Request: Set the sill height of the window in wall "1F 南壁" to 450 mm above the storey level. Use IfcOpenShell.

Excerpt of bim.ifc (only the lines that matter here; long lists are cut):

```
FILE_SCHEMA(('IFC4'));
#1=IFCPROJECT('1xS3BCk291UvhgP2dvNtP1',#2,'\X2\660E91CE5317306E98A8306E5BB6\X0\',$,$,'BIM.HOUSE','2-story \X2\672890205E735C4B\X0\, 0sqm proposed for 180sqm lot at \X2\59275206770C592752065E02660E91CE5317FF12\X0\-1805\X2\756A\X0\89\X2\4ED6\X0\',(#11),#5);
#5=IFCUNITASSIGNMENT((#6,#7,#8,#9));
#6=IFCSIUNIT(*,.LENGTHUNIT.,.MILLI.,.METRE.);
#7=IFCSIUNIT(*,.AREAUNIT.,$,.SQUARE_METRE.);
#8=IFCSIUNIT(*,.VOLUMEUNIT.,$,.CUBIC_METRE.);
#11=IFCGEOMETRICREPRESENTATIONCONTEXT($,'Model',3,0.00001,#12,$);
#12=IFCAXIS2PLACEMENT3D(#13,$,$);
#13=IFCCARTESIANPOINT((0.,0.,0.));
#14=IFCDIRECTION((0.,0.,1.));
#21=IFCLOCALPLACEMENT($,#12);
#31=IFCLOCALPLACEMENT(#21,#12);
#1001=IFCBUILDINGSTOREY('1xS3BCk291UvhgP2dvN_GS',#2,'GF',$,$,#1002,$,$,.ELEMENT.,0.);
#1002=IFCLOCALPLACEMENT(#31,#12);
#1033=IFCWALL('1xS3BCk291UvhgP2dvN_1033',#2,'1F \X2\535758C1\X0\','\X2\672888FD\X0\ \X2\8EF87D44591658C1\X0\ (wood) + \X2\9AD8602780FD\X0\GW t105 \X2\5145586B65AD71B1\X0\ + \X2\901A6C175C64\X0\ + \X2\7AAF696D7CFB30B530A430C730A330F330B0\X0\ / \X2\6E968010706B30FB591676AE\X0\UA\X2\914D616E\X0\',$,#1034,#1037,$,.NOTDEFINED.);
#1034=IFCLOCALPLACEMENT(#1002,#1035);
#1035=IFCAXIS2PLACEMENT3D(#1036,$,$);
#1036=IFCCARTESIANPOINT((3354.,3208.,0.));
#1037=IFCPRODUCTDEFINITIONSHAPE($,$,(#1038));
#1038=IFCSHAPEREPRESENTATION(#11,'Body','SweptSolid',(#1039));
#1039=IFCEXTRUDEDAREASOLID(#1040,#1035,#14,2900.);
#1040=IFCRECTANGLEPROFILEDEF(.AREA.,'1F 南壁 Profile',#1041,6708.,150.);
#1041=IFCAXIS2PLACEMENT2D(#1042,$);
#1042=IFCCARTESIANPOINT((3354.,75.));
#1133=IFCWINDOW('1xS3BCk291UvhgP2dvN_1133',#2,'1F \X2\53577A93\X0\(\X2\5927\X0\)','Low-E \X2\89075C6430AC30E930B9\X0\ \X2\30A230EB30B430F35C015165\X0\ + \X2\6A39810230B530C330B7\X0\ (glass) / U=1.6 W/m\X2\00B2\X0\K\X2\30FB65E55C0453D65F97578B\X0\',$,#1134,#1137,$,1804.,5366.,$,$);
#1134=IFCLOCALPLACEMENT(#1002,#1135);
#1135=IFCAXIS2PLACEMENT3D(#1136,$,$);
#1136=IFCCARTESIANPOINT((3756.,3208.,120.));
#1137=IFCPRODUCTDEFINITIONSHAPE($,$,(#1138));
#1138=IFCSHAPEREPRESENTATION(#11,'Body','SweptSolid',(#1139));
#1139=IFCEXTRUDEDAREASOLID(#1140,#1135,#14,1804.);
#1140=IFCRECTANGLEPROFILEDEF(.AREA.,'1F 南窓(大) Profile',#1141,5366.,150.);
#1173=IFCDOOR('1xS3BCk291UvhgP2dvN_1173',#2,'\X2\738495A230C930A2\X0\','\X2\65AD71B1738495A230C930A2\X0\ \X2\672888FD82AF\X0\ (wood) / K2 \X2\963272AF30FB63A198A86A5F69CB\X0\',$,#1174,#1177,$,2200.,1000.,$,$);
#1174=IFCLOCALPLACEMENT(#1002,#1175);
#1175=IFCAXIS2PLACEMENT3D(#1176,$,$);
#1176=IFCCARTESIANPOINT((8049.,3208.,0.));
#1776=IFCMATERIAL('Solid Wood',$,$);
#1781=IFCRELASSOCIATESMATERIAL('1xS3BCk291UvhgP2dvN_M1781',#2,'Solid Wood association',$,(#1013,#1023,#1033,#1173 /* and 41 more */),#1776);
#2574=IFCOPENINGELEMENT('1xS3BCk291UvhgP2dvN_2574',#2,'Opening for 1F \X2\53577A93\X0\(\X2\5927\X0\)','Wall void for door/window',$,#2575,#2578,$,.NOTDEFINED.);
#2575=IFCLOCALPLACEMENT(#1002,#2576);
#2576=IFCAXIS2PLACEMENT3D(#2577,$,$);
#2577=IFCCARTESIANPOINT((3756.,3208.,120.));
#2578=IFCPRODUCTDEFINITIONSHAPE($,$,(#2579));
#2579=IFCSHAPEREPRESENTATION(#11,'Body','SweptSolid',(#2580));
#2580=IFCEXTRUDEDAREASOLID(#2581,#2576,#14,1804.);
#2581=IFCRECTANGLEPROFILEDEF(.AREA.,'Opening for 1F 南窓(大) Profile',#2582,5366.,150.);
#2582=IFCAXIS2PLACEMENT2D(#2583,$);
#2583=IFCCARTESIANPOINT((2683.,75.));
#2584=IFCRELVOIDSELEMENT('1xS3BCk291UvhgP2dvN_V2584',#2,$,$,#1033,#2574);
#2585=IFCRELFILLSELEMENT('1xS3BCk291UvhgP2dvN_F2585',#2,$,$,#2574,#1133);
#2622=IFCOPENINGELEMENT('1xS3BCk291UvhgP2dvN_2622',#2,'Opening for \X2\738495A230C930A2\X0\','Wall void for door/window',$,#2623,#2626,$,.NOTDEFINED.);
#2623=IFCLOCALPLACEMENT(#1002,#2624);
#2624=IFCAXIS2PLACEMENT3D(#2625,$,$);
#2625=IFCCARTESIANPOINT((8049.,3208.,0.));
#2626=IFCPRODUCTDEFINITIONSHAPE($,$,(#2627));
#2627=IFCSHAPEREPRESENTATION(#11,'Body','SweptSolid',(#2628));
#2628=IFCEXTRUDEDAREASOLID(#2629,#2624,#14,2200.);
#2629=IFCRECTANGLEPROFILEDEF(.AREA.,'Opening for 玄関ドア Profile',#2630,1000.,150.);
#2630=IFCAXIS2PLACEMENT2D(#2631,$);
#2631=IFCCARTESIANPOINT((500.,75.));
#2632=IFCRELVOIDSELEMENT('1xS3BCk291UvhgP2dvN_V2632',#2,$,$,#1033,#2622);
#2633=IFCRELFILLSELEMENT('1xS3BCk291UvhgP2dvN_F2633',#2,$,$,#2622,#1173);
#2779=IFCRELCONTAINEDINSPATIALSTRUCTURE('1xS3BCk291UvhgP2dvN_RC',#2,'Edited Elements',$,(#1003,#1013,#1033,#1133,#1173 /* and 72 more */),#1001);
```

```python
import numpy as np
import ifcopenshell
import ifcopenshell.api.geometry
import ifcopenshell.geom
import ifcopenshell.util.element
import ifcopenshell.util.placement
import ifcopenshell.util.shape
import ifcopenshell.util.unit

model = ifcopenshell.open("bim.ifc")
unit_scale = ifcopenshell.util.unit.calculate_unit_scale(model)

window = model.by_guid("1xS3BCk291UvhgP2dvN_1133")
opening = window.FillsVoids[0].RelatingOpeningElement
storey = ifcopenshell.util.element.get_container(window, ifc_class="IfcBuildingStorey")
level = ifcopenshell.util.placement.get_local_placement(storey.ObjectPlacement)[2, 3]

# The opening's origin need not be at the sill, so measure its lowest point.
shape = ifcopenshell.geom.create_shape(ifcopenshell.geom.settings(), opening)
bottom = ifcopenshell.util.shape.get_shape_bottom_elevation(shape, shape.geometry) / unit_scale
dz = level + 450.0 - bottom

shift = np.array([0.0, 0.0, dz])
# The window is not placed relative to its opening, so move both.
for product in (opening, window):
    matrix = ifcopenshell.util.placement.get_local_placement(product.ObjectPlacement)
    matrix[:3, 3] += shift
    ifcopenshell.api.geometry.edit_object_placement(model, product=product, matrix=matrix, is_si=False)

print(f"moved by {dz * unit_scale:+.3f} m")

model.write("bim_rev.ifc")
```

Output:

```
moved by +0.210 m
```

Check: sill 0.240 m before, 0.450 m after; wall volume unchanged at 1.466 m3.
